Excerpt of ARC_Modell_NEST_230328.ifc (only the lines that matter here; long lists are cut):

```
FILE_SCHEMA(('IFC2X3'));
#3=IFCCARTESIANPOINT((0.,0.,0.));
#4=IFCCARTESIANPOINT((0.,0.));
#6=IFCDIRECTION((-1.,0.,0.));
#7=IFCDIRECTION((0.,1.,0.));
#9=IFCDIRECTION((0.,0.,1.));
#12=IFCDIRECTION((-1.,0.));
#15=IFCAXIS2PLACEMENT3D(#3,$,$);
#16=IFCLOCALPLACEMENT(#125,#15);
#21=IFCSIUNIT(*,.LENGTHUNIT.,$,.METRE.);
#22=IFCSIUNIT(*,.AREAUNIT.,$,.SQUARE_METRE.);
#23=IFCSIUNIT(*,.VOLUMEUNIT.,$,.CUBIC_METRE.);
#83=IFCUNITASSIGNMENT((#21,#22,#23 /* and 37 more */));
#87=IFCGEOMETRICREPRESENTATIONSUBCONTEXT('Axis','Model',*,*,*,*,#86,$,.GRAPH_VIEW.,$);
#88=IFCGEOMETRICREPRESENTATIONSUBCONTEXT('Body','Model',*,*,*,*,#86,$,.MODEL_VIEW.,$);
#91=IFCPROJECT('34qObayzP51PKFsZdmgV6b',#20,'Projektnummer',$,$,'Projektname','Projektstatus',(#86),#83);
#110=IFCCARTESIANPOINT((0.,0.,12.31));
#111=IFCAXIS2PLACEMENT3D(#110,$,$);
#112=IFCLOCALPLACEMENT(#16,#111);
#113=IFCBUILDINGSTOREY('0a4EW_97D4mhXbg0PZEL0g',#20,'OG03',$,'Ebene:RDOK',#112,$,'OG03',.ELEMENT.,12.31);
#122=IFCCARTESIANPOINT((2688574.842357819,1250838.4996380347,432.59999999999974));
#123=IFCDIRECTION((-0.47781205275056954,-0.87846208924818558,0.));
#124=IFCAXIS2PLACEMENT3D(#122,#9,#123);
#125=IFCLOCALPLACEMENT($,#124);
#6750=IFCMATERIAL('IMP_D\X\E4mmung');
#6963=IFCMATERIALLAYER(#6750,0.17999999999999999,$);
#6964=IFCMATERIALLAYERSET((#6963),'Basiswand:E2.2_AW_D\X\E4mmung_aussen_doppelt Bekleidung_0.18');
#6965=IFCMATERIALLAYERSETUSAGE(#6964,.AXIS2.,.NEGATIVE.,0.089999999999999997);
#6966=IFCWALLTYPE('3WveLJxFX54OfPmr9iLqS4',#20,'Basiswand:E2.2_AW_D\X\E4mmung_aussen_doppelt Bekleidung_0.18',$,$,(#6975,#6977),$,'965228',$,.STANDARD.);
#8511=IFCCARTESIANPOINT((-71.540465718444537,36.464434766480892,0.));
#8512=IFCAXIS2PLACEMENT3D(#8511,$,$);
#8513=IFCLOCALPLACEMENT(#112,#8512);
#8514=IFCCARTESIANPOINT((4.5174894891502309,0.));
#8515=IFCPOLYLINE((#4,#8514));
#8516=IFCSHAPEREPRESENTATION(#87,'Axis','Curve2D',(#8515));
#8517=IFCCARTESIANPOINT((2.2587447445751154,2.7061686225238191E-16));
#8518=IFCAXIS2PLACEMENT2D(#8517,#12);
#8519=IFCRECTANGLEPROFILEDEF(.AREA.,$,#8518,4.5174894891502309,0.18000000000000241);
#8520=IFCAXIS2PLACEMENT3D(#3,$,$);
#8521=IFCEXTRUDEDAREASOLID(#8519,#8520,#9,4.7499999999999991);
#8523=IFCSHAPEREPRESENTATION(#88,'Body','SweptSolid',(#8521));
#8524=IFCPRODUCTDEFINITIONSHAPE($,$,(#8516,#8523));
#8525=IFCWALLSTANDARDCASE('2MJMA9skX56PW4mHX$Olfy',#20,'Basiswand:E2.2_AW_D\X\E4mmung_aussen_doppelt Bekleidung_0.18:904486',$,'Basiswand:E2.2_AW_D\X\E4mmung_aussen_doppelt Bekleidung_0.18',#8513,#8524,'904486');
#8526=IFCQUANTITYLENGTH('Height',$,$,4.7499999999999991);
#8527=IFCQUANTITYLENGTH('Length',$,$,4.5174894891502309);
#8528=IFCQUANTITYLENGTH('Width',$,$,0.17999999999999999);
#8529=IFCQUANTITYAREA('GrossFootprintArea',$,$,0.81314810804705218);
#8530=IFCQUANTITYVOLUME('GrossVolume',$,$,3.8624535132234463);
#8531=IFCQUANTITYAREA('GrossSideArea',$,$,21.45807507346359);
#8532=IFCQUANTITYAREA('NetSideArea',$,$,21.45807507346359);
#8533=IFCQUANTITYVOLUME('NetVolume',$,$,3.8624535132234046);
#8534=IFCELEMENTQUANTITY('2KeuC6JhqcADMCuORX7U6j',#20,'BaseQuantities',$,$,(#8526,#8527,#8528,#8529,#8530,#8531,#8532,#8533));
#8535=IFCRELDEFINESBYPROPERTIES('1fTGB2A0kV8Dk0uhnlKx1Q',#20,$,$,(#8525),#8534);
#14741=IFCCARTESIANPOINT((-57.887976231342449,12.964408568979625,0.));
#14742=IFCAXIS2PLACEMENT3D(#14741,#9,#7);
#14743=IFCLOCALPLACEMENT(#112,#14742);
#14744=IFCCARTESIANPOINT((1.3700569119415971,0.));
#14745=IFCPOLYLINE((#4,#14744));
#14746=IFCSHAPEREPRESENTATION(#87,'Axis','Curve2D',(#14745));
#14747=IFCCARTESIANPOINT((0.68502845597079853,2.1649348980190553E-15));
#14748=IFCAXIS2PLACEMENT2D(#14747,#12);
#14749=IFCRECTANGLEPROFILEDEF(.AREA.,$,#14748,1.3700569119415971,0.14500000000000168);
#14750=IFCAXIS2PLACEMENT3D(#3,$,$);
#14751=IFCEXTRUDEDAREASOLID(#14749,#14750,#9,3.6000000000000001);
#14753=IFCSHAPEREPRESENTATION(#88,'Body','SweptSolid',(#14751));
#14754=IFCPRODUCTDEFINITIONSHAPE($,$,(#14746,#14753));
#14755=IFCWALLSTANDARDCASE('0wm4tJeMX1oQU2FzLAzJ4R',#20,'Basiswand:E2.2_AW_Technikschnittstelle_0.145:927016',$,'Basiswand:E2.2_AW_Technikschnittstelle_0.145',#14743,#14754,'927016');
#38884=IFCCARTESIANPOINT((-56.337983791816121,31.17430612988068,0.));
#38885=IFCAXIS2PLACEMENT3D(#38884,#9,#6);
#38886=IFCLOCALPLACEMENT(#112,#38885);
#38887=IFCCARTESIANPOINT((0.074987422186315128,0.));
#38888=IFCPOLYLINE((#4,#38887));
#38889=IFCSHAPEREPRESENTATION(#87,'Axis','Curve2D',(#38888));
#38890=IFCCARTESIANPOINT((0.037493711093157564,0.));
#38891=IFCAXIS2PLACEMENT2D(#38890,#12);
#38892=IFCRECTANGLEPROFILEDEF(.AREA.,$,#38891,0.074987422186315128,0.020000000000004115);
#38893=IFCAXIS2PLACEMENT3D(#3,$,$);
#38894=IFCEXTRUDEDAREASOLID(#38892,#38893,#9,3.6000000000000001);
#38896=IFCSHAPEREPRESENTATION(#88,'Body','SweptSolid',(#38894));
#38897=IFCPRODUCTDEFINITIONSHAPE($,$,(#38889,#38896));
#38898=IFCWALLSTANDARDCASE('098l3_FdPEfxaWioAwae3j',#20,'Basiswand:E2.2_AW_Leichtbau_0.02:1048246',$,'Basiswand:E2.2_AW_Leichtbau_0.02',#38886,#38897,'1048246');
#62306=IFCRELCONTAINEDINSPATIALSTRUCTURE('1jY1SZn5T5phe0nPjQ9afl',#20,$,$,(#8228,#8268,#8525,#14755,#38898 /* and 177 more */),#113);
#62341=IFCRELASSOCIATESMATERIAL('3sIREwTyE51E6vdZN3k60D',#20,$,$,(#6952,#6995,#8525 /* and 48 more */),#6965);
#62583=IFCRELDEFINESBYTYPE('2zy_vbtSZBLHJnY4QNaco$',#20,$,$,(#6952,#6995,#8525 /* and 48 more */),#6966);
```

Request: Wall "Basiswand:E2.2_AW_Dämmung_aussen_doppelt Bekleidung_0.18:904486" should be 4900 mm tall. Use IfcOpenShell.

```python
import ifcopenshell
import ifcopenshell.api.pset
import ifcopenshell.geom
import ifcopenshell.util.element
import ifcopenshell.util.representation
import ifcopenshell.util.shape
import ifcopenshell.util.unit

model = ifcopenshell.open("ARC_Modell_NEST_230328.ifc")
unit_scale = ifcopenshell.util.unit.calculate_unit_scale(model)
area_scale = ifcopenshell.util.unit.calculate_unit_scale(model, "AREAUNIT")
volume_scale = ifcopenshell.util.unit.calculate_unit_scale(model, "VOLUMEUNIT")
settings = ifcopenshell.geom.settings()


def volume(element):
    """Net volume in cubic metres, openings subtracted."""
    shape = ifcopenshell.geom.create_shape(settings, element)
    return ifcopenshell.util.shape.get_volume(shape.geometry)


wall = model.by_guid("2MJMA9skX56PW4mHX$Olfy")
before = volume(wall)

body = ifcopenshell.util.representation.get_representation(wall, "Model", "Body")
solid = body.Items[0]
old_height = solid.Depth
solid.Depth = 4.9
after = volume(wall)
thickness = 0.18  # wall thickness in metres

# Update the stored height, areas and volumes.
qto = model.by_id(ifcopenshell.util.element.get_pset(wall, "BaseQuantities", should_inherit=False)["id"])
ifcopenshell.api.pset.edit_qto(model, qto=qto, properties={
    "Height": solid.Depth,
    "GrossVolume": ifcopenshell.util.element.get_pset(wall, "BaseQuantities", "GrossVolume") * solid.Depth / old_height,
    "GrossSideArea": ifcopenshell.util.element.get_pset(wall, "BaseQuantities", "GrossSideArea") * solid.Depth / old_height,
    "NetSideArea": after / thickness / area_scale,
    "NetVolume": after / volume_scale,
})

print(f"height {old_height:g} -> {solid.Depth:g}, volume {before:.3f} -> {after:.3f} m3")

model.write("ARC_Modell_NEST_230328_rev.ifc")
```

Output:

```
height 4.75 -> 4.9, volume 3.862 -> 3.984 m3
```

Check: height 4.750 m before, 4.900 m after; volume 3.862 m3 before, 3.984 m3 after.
